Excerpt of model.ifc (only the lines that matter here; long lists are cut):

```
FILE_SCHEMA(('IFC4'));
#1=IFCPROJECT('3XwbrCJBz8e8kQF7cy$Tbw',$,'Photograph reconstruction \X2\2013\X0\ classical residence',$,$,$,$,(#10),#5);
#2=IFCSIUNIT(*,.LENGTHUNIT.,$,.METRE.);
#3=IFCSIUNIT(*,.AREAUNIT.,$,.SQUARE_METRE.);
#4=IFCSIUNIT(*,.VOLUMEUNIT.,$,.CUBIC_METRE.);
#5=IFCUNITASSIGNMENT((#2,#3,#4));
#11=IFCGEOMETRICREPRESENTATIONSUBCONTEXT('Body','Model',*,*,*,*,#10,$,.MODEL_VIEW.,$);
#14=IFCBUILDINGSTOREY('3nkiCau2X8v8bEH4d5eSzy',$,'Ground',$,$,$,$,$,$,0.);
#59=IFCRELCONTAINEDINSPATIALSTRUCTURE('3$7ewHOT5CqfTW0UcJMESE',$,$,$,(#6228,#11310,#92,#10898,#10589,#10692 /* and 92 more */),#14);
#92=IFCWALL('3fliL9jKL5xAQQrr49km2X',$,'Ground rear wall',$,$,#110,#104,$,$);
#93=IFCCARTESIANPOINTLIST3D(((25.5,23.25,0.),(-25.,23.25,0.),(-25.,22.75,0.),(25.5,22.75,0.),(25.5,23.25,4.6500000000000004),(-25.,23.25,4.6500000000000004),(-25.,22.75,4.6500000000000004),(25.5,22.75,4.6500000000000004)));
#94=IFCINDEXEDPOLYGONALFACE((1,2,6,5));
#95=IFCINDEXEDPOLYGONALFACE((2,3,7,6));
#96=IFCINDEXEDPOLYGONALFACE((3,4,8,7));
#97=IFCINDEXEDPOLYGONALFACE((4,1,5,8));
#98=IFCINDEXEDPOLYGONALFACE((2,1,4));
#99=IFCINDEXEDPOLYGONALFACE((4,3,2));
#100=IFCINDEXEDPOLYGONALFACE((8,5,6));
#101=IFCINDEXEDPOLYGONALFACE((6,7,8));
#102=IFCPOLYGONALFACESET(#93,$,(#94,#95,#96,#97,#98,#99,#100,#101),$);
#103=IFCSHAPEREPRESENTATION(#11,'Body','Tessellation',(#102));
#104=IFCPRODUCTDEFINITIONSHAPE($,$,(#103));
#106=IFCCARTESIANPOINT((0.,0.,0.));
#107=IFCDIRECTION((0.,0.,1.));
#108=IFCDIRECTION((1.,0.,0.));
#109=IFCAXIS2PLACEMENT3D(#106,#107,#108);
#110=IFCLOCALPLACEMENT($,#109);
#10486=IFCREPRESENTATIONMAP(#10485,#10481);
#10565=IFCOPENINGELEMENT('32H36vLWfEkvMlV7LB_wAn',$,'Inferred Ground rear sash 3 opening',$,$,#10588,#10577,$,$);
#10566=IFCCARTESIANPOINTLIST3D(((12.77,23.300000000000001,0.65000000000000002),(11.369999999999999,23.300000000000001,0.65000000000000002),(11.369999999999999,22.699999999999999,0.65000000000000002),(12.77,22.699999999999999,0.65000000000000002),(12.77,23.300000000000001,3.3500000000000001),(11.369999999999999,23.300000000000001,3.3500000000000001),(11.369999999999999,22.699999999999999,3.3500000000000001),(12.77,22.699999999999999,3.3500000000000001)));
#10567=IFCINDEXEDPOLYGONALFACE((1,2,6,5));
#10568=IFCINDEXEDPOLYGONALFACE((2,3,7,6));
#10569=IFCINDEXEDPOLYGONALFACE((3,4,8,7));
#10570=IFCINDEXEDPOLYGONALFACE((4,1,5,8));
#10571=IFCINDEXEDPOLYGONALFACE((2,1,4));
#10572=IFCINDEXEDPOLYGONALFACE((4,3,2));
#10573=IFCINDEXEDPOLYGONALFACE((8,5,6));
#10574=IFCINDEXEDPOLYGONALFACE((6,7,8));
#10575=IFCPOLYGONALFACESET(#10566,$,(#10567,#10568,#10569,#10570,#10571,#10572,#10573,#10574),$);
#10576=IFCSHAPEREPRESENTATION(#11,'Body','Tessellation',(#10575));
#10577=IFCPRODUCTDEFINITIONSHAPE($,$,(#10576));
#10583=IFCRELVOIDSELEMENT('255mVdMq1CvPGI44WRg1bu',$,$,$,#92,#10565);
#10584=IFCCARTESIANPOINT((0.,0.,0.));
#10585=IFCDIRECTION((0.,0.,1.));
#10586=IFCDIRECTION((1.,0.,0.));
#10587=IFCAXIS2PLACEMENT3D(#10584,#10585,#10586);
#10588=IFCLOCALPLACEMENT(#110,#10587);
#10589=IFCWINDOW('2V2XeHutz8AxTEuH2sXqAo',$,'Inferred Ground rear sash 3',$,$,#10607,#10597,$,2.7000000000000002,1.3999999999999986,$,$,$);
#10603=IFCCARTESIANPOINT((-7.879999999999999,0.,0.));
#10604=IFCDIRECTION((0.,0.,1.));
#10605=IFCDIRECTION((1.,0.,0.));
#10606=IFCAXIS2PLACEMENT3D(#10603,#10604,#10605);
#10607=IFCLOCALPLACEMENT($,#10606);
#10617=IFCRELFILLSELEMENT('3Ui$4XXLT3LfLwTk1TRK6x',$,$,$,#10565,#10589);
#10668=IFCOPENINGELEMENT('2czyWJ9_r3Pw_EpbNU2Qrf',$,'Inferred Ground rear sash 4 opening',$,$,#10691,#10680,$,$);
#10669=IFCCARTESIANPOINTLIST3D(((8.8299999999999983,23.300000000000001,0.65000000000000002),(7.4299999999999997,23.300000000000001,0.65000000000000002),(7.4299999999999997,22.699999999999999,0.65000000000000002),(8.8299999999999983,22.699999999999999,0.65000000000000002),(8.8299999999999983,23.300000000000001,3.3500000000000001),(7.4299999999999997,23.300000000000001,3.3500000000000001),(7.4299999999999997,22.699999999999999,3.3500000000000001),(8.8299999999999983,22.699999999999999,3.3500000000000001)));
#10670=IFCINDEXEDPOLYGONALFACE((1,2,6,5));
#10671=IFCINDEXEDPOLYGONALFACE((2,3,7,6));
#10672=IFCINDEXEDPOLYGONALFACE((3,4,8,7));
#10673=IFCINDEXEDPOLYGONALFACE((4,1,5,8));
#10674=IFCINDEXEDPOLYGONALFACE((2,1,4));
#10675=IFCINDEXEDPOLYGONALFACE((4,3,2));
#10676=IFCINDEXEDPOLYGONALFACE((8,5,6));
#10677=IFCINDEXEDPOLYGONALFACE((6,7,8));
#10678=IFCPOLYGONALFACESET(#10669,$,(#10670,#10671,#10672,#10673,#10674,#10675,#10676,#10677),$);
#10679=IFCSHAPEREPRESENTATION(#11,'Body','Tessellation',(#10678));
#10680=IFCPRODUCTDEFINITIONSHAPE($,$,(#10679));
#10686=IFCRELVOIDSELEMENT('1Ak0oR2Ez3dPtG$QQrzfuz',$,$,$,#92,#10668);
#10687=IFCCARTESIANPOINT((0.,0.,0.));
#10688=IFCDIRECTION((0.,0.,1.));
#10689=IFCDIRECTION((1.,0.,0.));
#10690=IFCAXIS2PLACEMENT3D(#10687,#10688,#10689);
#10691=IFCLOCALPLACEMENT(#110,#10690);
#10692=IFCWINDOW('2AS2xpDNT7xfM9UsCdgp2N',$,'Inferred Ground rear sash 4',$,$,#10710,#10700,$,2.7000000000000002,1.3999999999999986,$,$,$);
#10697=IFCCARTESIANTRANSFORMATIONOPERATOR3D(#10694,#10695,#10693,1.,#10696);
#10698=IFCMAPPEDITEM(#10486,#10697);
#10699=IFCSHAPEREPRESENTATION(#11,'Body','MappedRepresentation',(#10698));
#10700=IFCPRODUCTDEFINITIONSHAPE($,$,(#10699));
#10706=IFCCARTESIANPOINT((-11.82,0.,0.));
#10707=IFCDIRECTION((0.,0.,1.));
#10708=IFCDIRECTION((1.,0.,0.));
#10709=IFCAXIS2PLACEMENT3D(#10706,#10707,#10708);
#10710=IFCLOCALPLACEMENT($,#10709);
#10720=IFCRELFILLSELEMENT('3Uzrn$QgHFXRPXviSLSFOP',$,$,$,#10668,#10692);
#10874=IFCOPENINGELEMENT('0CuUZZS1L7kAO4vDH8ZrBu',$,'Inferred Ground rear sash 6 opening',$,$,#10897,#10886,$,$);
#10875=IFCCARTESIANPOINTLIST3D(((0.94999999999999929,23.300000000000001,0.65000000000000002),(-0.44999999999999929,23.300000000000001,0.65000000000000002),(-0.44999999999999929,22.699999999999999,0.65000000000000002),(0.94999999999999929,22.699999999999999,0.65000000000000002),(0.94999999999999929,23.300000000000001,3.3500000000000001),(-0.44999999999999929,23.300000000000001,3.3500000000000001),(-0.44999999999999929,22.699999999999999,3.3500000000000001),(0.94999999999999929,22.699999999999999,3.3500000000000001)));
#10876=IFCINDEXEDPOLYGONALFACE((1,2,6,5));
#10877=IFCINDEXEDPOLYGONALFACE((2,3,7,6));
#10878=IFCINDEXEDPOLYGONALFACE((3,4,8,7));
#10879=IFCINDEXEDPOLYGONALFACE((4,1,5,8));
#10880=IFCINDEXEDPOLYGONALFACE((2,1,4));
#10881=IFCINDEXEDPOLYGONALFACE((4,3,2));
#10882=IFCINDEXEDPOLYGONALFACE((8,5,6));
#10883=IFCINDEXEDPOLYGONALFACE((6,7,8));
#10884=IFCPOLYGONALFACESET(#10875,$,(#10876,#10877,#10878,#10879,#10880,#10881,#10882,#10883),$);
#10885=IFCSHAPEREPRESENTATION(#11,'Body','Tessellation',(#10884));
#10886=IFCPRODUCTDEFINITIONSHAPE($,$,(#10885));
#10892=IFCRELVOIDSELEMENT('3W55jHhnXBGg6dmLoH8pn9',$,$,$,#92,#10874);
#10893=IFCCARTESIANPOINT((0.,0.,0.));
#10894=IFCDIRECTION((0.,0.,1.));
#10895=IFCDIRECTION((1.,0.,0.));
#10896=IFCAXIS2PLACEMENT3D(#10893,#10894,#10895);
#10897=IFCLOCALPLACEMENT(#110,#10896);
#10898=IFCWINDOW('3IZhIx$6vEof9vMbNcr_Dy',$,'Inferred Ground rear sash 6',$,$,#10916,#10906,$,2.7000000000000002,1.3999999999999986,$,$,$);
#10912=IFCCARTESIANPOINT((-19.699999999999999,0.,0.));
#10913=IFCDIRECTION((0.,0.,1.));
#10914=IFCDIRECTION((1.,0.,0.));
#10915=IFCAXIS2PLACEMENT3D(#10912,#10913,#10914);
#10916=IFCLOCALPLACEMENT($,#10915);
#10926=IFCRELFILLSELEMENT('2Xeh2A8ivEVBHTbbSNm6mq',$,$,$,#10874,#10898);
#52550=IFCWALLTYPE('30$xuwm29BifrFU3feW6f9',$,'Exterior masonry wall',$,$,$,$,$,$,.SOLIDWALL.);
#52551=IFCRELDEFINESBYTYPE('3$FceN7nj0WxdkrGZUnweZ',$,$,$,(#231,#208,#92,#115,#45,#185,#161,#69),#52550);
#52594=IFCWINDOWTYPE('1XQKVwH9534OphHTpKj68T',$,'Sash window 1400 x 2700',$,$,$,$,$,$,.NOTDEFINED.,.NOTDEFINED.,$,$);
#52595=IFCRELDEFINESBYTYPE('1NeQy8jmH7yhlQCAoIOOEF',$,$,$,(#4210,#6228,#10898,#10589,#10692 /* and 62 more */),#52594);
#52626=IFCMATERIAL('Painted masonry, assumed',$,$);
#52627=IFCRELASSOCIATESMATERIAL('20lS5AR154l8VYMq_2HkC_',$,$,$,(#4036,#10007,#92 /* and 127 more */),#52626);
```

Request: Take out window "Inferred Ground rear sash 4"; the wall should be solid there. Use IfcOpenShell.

```python
import ifcopenshell
import ifcopenshell.api.feature
import ifcopenshell.api.root
import ifcopenshell.geom
import ifcopenshell.util.shape

model = ifcopenshell.open("model.ifc")
settings = ifcopenshell.geom.settings()


def volume(element):
    """Net volume in cubic metres, openings subtracted."""
    shape = ifcopenshell.geom.create_shape(settings, element)
    return ifcopenshell.util.shape.get_volume(shape.geometry)


window = model.by_guid("2AS2xpDNT7xfM9UsCdgp2N")
opening = window.FillsVoids[0].RelatingOpeningElement
wall = opening.VoidsElements[0].RelatingBuildingElement
before = volume(wall)

ifcopenshell.api.root.remove_product(model, product=window)
ifcopenshell.api.feature.remove_feature(model, feature=opening)

after = volume(wall)

print(f"wall volume {before:.3f} -> {after:.3f} m3")

model.write("model-out.ifc")
```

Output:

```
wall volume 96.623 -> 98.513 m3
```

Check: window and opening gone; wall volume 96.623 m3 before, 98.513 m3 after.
